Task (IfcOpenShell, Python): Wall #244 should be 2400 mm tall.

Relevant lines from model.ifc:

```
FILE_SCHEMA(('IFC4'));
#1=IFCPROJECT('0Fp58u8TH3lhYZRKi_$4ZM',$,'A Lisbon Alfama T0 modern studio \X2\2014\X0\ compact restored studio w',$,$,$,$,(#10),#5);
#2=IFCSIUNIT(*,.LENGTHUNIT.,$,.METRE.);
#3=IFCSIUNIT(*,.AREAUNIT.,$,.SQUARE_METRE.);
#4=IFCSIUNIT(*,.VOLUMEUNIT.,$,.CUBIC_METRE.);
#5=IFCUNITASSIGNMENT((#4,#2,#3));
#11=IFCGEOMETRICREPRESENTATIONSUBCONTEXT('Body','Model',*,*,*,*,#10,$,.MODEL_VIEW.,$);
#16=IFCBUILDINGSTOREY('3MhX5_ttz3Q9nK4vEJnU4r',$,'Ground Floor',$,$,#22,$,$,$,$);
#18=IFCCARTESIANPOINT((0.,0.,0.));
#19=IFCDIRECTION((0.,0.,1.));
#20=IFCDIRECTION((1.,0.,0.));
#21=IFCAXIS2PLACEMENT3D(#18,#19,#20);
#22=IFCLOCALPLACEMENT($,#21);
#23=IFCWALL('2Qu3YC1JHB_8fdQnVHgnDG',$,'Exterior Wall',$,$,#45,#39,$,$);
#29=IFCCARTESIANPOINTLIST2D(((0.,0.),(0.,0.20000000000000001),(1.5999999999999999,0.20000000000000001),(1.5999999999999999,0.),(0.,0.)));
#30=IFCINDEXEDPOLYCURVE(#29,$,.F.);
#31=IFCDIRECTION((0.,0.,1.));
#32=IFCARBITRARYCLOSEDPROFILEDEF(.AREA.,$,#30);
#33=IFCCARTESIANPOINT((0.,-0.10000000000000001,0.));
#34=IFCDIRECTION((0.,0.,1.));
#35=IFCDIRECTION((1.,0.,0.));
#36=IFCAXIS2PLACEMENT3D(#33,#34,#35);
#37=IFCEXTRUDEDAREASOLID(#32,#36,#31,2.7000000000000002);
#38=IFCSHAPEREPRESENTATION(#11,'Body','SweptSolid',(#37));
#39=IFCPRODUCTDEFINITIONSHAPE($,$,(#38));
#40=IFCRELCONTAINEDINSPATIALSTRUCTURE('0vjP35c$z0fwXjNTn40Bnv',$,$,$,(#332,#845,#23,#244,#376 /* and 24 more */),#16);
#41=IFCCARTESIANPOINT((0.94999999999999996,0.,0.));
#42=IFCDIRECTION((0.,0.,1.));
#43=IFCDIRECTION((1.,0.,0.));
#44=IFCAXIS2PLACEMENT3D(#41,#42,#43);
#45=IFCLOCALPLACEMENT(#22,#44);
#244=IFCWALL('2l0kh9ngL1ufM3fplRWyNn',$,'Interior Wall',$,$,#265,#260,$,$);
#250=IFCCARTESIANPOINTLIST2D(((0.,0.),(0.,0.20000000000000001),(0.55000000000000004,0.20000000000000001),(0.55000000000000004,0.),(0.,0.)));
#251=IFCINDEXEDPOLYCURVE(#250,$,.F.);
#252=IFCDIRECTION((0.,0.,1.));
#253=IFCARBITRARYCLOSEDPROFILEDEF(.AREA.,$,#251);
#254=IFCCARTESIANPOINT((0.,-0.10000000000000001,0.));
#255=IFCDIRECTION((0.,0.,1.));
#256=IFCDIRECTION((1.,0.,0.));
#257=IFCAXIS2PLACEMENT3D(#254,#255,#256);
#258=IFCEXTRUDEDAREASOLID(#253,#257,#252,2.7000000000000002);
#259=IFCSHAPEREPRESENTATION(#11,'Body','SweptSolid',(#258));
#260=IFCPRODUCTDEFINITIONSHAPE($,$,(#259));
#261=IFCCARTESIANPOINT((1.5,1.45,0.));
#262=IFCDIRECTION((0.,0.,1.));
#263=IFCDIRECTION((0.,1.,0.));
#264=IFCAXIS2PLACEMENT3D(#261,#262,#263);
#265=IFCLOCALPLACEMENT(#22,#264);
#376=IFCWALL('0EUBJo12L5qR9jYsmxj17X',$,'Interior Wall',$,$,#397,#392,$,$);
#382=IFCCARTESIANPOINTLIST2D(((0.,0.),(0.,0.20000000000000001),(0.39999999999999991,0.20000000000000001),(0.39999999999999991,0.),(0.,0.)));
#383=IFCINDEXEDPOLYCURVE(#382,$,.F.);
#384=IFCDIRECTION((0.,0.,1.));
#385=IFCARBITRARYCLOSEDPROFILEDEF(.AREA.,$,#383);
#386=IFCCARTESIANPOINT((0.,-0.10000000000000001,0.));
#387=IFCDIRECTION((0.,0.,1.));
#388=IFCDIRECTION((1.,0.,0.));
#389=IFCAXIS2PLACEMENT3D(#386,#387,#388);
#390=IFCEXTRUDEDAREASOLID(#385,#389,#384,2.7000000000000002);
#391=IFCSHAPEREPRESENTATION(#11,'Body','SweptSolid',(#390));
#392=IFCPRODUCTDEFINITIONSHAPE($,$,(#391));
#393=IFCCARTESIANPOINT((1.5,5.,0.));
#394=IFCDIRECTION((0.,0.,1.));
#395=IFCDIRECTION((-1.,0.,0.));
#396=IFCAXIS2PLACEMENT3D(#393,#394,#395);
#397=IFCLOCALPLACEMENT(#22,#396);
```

```python
import ifcopenshell
import ifcopenshell.geom
import ifcopenshell.util.representation
import ifcopenshell.util.shape
import ifcopenshell.util.unit

model = ifcopenshell.open("model.ifc")
unit_scale = ifcopenshell.util.unit.calculate_unit_scale(model)
settings = ifcopenshell.geom.settings()


def volume(element):
    """Net volume in cubic metres, openings subtracted."""
    shape = ifcopenshell.geom.create_shape(settings, element)
    return ifcopenshell.util.shape.get_volume(shape.geometry)


wall = model.by_id(244)
before = volume(wall)

body = ifcopenshell.util.representation.get_representation(wall, "Model", "Body")
solid = body.Items[0]
old_height = solid.Depth
solid.Depth = 2.4 / unit_scale
after = volume(wall)

print(f"height {old_height:g} -> {solid.Depth:g}, volume {before:.3f} -> {after:.3f} m3")

model.write("model-out.ifc")
```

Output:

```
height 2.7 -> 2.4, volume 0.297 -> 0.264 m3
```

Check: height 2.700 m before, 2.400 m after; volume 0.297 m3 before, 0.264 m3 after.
